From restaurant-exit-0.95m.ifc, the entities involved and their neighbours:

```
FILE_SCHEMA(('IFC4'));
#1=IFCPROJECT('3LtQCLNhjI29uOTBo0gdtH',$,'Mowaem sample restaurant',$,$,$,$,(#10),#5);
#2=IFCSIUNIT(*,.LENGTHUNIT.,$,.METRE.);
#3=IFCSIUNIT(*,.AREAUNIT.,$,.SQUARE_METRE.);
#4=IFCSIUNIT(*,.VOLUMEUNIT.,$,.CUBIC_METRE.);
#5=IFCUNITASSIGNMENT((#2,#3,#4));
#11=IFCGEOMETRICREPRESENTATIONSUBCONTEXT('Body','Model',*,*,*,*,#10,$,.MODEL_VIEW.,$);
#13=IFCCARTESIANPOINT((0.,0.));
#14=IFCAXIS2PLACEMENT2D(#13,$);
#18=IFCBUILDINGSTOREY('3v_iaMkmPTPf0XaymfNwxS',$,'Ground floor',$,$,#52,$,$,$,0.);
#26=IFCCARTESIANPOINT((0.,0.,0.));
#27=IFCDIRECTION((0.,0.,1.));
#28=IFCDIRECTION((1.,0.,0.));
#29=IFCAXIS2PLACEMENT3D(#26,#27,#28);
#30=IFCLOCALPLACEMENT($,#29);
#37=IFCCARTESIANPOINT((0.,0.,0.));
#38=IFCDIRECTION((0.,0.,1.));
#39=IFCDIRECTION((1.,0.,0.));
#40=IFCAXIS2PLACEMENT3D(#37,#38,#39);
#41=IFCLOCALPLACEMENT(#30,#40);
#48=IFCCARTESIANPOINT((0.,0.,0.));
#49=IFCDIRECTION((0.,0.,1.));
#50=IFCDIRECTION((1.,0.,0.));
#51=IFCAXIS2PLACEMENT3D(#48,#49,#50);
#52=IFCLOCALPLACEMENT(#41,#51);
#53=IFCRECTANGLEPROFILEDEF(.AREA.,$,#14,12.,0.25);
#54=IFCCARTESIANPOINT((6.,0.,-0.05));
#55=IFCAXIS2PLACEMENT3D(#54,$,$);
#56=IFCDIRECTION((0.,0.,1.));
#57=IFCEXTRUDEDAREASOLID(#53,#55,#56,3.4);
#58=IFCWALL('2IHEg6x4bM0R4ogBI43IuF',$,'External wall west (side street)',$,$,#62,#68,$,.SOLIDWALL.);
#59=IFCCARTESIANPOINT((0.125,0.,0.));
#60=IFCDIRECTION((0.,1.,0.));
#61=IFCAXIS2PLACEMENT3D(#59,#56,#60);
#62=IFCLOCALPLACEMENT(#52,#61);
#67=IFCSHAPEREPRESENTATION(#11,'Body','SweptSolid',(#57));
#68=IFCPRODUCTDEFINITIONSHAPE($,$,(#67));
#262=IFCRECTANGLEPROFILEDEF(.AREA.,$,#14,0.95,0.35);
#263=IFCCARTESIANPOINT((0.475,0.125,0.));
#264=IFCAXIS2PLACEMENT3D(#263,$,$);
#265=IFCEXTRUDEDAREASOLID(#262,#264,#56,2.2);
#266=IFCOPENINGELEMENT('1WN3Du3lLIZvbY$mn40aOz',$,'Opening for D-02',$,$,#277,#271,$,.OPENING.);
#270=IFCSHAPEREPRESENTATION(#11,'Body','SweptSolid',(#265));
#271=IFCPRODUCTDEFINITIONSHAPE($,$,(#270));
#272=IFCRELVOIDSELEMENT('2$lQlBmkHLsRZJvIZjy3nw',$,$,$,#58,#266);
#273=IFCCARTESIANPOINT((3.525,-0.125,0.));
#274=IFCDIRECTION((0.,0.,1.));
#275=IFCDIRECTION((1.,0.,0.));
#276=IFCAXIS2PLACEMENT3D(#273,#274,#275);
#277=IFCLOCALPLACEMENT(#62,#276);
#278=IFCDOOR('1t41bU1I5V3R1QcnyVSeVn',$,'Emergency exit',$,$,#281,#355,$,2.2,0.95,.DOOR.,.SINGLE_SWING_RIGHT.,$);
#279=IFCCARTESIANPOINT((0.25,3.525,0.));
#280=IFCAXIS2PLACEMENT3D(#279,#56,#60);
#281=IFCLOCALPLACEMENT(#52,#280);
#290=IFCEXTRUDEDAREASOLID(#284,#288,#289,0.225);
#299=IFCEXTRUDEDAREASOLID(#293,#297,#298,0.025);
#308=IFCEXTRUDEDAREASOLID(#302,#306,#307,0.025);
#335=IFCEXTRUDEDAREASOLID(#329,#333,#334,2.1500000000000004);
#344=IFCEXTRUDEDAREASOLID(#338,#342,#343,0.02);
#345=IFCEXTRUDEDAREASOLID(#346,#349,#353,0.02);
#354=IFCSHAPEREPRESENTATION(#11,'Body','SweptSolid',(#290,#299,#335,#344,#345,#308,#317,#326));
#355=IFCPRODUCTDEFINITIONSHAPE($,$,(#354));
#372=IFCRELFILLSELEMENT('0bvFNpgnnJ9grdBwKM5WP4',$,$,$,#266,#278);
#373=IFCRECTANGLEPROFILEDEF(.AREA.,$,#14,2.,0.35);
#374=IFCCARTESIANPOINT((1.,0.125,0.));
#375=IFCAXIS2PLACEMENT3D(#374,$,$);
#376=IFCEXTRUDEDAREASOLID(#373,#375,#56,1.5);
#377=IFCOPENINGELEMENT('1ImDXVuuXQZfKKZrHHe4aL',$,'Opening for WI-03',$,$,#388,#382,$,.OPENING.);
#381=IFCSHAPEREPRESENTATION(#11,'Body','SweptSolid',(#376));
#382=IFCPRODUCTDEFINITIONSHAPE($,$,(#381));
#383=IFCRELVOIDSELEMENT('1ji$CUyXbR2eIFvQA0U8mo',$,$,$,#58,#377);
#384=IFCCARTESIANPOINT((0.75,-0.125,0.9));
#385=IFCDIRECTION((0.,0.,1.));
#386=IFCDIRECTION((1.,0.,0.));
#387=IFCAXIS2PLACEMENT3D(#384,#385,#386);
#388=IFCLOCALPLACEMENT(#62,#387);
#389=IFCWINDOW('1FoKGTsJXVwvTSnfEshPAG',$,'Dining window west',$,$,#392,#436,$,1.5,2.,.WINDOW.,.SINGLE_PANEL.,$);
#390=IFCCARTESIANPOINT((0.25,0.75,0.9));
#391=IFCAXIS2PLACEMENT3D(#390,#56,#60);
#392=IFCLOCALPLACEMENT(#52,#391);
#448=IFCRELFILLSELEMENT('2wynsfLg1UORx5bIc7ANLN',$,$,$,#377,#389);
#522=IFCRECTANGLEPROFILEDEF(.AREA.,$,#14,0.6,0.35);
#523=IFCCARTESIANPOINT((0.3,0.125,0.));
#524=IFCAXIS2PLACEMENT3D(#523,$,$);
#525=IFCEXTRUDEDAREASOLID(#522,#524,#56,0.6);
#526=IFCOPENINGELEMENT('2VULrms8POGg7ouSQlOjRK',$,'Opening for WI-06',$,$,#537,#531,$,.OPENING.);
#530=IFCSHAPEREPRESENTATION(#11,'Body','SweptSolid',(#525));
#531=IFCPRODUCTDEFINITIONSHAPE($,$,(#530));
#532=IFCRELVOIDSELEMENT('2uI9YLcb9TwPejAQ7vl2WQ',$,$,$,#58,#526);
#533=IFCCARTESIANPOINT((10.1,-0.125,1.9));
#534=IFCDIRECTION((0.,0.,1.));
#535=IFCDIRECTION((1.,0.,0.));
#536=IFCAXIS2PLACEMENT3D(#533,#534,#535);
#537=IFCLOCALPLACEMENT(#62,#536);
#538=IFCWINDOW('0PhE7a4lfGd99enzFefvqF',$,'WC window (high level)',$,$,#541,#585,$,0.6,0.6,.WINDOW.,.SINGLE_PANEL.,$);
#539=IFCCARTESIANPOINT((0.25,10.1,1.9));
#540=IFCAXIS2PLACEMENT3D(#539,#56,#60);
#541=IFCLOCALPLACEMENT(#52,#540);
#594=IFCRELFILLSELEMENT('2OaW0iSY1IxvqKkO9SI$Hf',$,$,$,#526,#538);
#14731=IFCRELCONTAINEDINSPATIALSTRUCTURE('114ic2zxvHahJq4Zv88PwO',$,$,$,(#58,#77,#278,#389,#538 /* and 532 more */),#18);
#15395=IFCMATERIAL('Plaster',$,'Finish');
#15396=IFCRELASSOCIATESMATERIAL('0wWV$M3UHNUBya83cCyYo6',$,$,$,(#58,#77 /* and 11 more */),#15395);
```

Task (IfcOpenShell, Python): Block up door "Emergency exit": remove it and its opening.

```python
import ifcopenshell
import ifcopenshell.api.feature
import ifcopenshell.api.root
import ifcopenshell.geom
import ifcopenshell.util.shape

model = ifcopenshell.open("restaurant-exit-0.95m.ifc")
settings = ifcopenshell.geom.settings()


def volume(element):
    """Net volume in cubic metres, openings subtracted."""
    shape = ifcopenshell.geom.create_shape(settings, element)
    return ifcopenshell.util.shape.get_volume(shape.geometry)


door = model.by_guid("1t41bU1I5V3R1QcnyVSeVn")
opening = door.FillsVoids[0].RelatingOpeningElement
wall = opening.VoidsElements[0].RelatingBuildingElement
before = volume(wall)

ifcopenshell.api.root.remove_product(model, product=door)
ifcopenshell.api.feature.remove_feature(model, feature=opening)

after = volume(wall)

print(f"wall volume {before:.3f} -> {after:.3f} m3")

model.write("restaurant-exit-0.95m_v2.ifc")
```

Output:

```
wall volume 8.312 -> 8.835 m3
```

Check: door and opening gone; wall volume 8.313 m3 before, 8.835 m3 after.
